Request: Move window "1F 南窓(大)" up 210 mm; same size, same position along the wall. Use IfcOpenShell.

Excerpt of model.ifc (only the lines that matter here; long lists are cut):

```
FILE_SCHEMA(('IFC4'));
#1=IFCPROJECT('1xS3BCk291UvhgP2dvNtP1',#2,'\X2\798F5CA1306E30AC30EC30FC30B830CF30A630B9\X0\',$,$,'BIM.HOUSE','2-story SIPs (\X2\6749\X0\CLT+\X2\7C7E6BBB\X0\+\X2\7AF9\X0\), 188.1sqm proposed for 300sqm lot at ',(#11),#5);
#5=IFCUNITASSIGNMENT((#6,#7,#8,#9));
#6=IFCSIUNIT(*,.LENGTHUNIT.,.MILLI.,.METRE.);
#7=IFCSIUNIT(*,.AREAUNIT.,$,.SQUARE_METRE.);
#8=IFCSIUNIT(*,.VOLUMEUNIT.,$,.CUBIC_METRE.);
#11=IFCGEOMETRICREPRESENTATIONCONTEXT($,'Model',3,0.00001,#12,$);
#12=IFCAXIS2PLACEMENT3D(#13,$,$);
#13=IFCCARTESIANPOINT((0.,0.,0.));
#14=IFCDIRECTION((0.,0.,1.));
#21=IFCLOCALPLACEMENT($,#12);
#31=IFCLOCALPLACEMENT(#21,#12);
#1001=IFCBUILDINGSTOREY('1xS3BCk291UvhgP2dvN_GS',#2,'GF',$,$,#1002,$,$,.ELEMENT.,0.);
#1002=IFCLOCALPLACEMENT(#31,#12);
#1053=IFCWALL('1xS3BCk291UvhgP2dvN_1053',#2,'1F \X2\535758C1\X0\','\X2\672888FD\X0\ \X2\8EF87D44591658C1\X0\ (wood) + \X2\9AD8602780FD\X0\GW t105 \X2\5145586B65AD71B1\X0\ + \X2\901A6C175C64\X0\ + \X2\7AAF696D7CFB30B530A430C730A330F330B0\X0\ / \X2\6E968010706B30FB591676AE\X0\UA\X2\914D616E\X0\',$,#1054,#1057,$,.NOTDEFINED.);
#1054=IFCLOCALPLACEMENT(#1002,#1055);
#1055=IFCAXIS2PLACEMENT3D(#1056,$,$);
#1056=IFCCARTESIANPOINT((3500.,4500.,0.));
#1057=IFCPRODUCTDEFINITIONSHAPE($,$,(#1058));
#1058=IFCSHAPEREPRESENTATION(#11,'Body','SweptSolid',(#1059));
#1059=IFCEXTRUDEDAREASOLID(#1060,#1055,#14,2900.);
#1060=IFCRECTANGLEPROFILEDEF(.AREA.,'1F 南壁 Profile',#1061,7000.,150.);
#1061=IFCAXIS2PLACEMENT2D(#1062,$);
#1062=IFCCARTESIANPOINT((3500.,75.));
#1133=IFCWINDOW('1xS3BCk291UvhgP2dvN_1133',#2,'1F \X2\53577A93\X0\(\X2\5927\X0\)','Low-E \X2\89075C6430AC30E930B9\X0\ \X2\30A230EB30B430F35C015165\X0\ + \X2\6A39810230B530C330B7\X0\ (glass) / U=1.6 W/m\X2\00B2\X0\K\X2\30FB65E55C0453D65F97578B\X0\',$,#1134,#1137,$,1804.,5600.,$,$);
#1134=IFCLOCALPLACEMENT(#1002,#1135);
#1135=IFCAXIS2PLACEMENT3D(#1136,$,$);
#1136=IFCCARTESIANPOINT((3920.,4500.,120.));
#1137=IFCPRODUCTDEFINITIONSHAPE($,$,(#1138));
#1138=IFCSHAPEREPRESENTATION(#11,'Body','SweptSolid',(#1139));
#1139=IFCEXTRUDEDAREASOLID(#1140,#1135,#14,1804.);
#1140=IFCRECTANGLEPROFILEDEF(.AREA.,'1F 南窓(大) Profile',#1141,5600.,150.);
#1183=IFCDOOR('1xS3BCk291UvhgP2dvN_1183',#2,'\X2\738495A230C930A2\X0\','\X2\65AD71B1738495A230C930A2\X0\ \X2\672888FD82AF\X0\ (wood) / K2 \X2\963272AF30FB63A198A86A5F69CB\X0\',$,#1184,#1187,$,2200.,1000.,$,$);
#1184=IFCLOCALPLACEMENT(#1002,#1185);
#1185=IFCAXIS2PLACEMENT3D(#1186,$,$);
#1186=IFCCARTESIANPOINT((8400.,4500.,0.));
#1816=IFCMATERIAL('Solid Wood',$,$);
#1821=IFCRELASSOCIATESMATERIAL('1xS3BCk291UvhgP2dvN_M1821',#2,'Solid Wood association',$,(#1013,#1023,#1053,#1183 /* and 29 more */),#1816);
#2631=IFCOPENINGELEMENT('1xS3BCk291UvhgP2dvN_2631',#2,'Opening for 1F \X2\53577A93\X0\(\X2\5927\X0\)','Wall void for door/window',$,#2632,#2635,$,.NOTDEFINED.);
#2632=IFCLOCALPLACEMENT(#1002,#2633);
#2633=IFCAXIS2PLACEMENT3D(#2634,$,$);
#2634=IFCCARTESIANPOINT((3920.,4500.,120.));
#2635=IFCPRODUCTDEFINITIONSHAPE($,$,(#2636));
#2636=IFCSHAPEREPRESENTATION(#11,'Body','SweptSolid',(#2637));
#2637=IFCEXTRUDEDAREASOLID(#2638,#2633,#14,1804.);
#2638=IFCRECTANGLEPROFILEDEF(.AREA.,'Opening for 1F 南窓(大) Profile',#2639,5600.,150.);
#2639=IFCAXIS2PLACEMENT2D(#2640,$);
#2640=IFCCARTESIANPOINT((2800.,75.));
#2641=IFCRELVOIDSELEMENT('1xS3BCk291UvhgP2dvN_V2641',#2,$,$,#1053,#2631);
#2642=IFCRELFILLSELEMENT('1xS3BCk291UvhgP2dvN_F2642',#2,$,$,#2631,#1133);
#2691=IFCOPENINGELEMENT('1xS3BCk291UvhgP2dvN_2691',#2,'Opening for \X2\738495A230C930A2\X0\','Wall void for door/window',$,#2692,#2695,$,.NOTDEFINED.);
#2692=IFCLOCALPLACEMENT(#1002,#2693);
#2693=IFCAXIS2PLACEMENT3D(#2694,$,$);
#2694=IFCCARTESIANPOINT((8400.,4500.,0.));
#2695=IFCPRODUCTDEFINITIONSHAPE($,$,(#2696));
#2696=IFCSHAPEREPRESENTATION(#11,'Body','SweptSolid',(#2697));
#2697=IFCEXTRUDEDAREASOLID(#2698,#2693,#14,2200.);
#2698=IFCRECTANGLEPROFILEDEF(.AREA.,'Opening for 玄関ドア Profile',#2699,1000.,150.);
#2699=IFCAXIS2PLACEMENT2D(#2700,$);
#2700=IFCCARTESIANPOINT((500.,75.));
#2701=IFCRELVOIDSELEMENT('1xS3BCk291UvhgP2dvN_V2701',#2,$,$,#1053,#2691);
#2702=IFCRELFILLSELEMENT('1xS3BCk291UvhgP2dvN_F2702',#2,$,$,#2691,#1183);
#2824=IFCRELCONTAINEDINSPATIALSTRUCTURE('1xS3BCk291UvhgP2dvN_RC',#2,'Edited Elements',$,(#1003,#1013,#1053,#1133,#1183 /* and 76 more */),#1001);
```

```python
import numpy as np
import ifcopenshell
import ifcopenshell.api.geometry
import ifcopenshell.util.placement
import ifcopenshell.util.unit

model = ifcopenshell.open("model.ifc")
unit_scale = ifcopenshell.util.unit.calculate_unit_scale(model)

window = model.by_guid("1xS3BCk291UvhgP2dvN_1133")
opening = window.FillsVoids[0].RelatingOpeningElement
dz = 0.21 / unit_scale

shift = np.array([0.0, 0.0, dz])
# The window is not placed relative to its opening, so move both.
for product in (opening, window):
    matrix = ifcopenshell.util.placement.get_local_placement(product.ObjectPlacement)
    matrix[:3, 3] += shift
    ifcopenshell.api.geometry.edit_object_placement(model, product=product, matrix=matrix, is_si=False)

print(f"moved by {dz * unit_scale:+.3f} m")

model.write("model_edited.ifc")
```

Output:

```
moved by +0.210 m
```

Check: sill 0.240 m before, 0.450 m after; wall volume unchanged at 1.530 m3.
